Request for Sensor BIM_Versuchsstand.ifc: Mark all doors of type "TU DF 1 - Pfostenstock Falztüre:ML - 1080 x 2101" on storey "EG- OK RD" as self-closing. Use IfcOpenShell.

First a look at what the model holds.

```python
import ifcopenshell
import ifcopenshell.util.element

model = ifcopenshell.open("Sensor BIM_Versuchsstand.ifc")
print(model.schema)
storey = next(s for s in model.by_type("IfcBuildingStorey") if s.Name == "EG- OK RD")
doors = [e for e in ifcopenshell.util.element.get_decomposition(storey) if e.is_a("IfcDoor")]
seen = {}
for e in doors:
    element_type = ifcopenshell.util.element.get_type(e)
    key = (element_type.Name if element_type != e and element_type else None, ifcopenshell.util.element.get_pset(e, "Pset_DoorCommon", "SelfClosing"))
    seen[key] = seen.get(key, 0) + 1
for (name, value), count in sorted(seen.items(), key=str):
    print(count, "x", name, "|", value)
```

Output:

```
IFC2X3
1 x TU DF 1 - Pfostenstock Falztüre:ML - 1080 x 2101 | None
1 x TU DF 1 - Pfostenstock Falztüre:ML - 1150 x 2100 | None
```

```python
import ifcopenshell
import ifcopenshell.api.pset
import ifcopenshell.util.element

model = ifcopenshell.open("Sensor BIM_Versuchsstand.ifc")

storey = next(s for s in model.by_type("IfcBuildingStorey") if s.Name == "EG- OK RD")
doors = [e for e in ifcopenshell.util.element.get_decomposition(storey) if e.is_a("IfcDoor")]

count = 0
for e in doors:
    element_type = ifcopenshell.util.element.get_type(e)
    if element_type in (None, e) or element_type.Name != "TU DF 1 - Pfostenstock Falztüre:ML - 1080 x 2101":
        continue
    # add_pset returns the element's existing set when there is one.
    pset = ifcopenshell.api.pset.add_pset(model, product=e, name="Pset_DoorCommon")
    ifcopenshell.api.pset.edit_pset(model, pset=pset, properties={"SelfClosing": True})
    count += 1

print(count, "doors updated")

model.write("Sensor BIM_Versuchsstand_updated.ifc")
```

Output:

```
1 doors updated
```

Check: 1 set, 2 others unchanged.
